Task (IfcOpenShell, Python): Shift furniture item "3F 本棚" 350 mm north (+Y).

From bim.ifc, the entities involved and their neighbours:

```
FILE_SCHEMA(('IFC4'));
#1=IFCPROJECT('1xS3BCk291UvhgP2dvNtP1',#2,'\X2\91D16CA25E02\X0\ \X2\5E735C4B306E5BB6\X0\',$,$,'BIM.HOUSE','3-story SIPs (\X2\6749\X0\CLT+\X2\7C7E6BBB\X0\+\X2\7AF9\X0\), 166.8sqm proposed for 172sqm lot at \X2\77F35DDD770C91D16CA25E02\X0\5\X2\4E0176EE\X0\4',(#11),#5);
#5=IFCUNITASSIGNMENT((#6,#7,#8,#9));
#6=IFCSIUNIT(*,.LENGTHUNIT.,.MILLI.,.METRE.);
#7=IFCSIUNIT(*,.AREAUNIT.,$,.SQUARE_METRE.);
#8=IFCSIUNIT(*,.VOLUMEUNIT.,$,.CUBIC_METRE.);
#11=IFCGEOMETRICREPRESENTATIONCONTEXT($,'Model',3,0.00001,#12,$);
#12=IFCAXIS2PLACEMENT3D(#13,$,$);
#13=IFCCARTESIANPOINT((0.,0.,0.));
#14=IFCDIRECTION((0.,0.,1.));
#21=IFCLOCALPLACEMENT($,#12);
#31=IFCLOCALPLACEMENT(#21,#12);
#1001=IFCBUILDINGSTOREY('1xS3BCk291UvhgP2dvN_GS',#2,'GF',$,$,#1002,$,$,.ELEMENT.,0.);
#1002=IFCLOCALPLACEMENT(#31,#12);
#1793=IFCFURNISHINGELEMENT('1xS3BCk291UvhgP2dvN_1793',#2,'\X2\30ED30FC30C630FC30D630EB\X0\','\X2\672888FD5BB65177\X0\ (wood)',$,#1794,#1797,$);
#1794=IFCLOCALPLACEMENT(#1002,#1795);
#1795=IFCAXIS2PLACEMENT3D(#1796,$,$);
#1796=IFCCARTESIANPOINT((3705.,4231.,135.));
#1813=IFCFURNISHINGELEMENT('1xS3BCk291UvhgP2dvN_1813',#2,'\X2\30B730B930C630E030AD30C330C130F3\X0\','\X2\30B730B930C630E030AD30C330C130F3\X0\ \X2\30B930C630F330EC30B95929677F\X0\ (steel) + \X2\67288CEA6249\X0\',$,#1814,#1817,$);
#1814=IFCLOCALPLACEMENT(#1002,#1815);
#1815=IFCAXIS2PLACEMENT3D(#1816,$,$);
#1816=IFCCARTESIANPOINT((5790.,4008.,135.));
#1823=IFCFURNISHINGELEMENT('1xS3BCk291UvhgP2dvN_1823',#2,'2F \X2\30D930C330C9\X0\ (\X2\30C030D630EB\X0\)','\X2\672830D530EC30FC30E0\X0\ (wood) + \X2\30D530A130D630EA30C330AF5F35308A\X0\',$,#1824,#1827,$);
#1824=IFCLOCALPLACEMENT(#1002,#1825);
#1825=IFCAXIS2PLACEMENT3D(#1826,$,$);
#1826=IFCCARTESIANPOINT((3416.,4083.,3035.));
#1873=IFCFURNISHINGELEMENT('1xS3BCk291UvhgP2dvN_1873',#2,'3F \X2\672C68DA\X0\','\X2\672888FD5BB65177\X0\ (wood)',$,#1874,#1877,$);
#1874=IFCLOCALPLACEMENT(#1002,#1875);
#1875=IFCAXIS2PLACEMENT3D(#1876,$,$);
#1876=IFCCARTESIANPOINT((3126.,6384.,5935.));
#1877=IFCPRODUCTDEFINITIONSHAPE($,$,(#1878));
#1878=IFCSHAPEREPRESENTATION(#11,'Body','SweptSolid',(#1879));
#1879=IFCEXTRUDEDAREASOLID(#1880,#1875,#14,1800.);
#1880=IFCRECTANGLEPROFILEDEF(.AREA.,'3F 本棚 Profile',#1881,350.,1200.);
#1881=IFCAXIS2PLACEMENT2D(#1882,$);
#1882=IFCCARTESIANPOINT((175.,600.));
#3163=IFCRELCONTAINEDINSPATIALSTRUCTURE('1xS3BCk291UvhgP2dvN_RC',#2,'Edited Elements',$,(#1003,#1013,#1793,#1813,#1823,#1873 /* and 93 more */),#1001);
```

```python
import ifcopenshell
import ifcopenshell.api.geometry
import ifcopenshell.util.placement
import ifcopenshell.util.unit

model = ifcopenshell.open("bim.ifc")
unit_scale = ifcopenshell.util.unit.calculate_unit_scale(model)

item = model.by_guid("1xS3BCk291UvhgP2dvN_1873")
matrix = ifcopenshell.util.placement.get_local_placement(item.ObjectPlacement)
matrix[1, 3] += 0.35 / unit_scale
ifcopenshell.api.geometry.edit_object_placement(model, product=item, matrix=matrix, is_si=False)

print(ifcopenshell.util.placement.get_local_placement(item.ObjectPlacement).round(3) + 0.0)

model.write("bim_updated.ifc")
```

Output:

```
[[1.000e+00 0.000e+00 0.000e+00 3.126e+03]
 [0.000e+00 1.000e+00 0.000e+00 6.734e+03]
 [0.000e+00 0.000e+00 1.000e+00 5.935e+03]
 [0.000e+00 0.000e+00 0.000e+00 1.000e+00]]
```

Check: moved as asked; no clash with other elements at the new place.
